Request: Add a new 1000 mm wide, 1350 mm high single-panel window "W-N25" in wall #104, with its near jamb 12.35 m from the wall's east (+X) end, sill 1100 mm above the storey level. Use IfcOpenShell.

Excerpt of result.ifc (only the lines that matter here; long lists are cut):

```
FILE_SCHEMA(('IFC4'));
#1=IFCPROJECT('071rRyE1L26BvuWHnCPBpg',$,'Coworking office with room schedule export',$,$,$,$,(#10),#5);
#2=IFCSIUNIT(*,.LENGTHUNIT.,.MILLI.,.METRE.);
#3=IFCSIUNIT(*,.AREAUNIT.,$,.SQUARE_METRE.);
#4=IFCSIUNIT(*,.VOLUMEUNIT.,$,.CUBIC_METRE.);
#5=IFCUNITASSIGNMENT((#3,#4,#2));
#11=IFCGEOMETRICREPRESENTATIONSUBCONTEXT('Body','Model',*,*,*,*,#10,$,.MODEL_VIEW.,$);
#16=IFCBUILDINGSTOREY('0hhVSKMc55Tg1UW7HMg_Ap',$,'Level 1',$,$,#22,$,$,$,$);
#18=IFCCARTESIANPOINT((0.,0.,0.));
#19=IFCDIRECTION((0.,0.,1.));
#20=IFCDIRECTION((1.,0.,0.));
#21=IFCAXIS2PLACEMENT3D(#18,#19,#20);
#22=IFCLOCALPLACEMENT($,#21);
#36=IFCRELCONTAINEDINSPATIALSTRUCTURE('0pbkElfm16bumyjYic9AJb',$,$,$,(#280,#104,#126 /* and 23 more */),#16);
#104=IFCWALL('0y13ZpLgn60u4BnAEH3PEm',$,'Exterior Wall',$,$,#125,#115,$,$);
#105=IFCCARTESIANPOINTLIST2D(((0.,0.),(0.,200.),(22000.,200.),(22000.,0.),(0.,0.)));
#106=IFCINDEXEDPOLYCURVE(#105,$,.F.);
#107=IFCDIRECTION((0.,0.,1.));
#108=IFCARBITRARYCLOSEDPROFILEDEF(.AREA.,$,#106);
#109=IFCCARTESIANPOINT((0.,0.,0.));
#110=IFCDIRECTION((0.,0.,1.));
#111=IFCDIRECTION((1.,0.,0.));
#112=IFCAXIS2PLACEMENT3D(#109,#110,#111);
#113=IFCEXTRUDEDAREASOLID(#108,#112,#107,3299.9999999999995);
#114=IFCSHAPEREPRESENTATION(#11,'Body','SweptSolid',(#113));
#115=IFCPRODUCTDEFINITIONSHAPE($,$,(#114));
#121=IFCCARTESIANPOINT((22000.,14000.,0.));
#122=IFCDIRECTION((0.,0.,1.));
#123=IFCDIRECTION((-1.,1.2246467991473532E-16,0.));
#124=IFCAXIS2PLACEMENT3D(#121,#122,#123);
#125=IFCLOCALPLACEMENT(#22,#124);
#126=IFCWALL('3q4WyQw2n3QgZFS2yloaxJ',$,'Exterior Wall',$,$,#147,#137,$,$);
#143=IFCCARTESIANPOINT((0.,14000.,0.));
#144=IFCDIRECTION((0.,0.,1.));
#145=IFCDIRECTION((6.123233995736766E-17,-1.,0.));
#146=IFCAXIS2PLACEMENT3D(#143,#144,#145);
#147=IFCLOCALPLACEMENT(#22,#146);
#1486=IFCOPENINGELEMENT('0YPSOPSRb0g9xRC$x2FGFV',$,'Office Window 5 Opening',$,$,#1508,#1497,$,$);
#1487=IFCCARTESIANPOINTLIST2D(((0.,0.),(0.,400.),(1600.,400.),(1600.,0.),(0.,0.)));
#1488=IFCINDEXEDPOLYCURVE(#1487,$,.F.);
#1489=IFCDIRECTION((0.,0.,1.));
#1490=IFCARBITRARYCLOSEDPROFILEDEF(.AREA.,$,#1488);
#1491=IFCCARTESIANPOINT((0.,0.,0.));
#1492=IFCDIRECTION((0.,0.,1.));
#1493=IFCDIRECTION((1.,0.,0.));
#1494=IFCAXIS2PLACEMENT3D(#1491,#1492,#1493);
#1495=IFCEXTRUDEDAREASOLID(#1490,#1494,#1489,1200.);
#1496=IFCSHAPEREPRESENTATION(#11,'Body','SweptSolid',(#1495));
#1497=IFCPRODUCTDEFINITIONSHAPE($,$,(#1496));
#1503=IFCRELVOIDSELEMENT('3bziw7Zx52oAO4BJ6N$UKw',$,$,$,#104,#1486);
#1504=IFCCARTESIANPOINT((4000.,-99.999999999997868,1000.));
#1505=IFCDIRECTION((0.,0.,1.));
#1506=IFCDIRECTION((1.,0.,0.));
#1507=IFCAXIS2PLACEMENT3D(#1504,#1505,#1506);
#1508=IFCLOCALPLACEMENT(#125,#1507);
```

```python
import numpy as np
import ifcopenshell
import ifcopenshell.api.feature
import ifcopenshell.api.geometry
import ifcopenshell.api.root
import ifcopenshell.api.spatial
import ifcopenshell.geom
import ifcopenshell.util.element
import ifcopenshell.util.placement
import ifcopenshell.util.representation
import ifcopenshell.util.shape
import ifcopenshell.util.unit

model = ifcopenshell.open("result.ifc")
unit_scale = ifcopenshell.util.unit.calculate_unit_scale(model)
settings = ifcopenshell.geom.settings()


def volume(element):
    """Net volume in cubic metres, openings subtracted."""
    shape = ifcopenshell.geom.create_shape(settings, element)
    return ifcopenshell.util.shape.get_volume(shape.geometry)


wall = model.by_guid("0y13ZpLgn60u4BnAEH3PEm")
storey = ifcopenshell.util.element.get_container(wall, ifc_class="IfcBuildingStorey")
context = ifcopenshell.util.representation.get_context(model, "Model", "Body", "MODEL_VIEW")
before = volume(wall)

width, height, from_end, sill = 1, 1.35, 12.35, 1.1  # metres

# The wall runs along its own X axis, and the end named is its -X end.
wall_shape = ifcopenshell.geom.create_shape(settings, wall)
x, y, z = ifcopenshell.util.shape.get_vertices(wall_shape.geometry).T
start = x.min() + from_end
face, thickness = float(y.min()), float(y.max() - y.min())
wall_matrix = ifcopenshell.util.placement.get_local_placement(wall.ObjectPlacement)
level = ifcopenshell.util.placement.get_local_placement(storey.ObjectPlacement)[2, 3]


def in_wall(x, y):
    """Placement at x, y metres in the wall's axes, at sill height."""
    matrix = wall_matrix.copy()
    matrix[:, 3] = wall_matrix @ np.array([x / unit_scale, y / unit_scale, 0.0, 1.0])
    matrix[2, 3] = level + sill / unit_scale
    return matrix


# Opening: a box that overshoots both wall faces by 50 mm.
opening = ifcopenshell.api.root.create_entity(model, ifc_class="IfcOpeningElement", predefined_type="OPENING")
box = ifcopenshell.api.geometry.add_wall_representation(
    model, context=context, length=width, height=height, thickness=thickness + 0.1
)
ifcopenshell.api.geometry.assign_representation(model, product=opening, representation=box)
ifcopenshell.api.geometry.edit_object_placement(model, product=opening, matrix=in_wall(start, face - 0.05), is_si=False)
ifcopenshell.api.feature.add_feature(model, feature=opening, element=wall)

window = ifcopenshell.api.root.create_entity(model, ifc_class="IfcWindow", name="W-N25", predefined_type="WINDOW")
window.OverallWidth, window.OverallHeight = width / unit_scale, height / unit_scale
window.PartitioningType = "SINGLE_PANEL"
body = ifcopenshell.api.geometry.add_window_representation(
    model,
    context=context,
    overall_width=window.OverallWidth,
    overall_height=window.OverallHeight,
    partition_type="SINGLE_PANEL",
)
ifcopenshell.api.geometry.assign_representation(model, product=window, representation=body)
ifcopenshell.api.spatial.assign_container(model, products=[window], relating_structure=storey)
ifcopenshell.api.feature.add_filling(model, opening=opening, element=window)

# Centre the window in the wall's thickness.
ifcopenshell.api.geometry.edit_object_placement(model, product=window, matrix=in_wall(start, face), is_si=False)
window_shape = ifcopenshell.geom.create_shape(settings, window)
depth = ifcopenshell.util.shape.get_vertices(window_shape.geometry)[:, 1]
offset = face + thickness / 2 - (depth.min() + depth.max()) / 2
ifcopenshell.api.geometry.edit_object_placement(model, product=window, matrix=in_wall(start, offset), is_si=False)

after = volume(wall)

print(f"wall volume {before:.3f} -> {after:.3f} m3")

model.write("result_rev.ifc")
```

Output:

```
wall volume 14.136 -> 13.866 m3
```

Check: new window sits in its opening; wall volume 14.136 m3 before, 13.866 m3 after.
